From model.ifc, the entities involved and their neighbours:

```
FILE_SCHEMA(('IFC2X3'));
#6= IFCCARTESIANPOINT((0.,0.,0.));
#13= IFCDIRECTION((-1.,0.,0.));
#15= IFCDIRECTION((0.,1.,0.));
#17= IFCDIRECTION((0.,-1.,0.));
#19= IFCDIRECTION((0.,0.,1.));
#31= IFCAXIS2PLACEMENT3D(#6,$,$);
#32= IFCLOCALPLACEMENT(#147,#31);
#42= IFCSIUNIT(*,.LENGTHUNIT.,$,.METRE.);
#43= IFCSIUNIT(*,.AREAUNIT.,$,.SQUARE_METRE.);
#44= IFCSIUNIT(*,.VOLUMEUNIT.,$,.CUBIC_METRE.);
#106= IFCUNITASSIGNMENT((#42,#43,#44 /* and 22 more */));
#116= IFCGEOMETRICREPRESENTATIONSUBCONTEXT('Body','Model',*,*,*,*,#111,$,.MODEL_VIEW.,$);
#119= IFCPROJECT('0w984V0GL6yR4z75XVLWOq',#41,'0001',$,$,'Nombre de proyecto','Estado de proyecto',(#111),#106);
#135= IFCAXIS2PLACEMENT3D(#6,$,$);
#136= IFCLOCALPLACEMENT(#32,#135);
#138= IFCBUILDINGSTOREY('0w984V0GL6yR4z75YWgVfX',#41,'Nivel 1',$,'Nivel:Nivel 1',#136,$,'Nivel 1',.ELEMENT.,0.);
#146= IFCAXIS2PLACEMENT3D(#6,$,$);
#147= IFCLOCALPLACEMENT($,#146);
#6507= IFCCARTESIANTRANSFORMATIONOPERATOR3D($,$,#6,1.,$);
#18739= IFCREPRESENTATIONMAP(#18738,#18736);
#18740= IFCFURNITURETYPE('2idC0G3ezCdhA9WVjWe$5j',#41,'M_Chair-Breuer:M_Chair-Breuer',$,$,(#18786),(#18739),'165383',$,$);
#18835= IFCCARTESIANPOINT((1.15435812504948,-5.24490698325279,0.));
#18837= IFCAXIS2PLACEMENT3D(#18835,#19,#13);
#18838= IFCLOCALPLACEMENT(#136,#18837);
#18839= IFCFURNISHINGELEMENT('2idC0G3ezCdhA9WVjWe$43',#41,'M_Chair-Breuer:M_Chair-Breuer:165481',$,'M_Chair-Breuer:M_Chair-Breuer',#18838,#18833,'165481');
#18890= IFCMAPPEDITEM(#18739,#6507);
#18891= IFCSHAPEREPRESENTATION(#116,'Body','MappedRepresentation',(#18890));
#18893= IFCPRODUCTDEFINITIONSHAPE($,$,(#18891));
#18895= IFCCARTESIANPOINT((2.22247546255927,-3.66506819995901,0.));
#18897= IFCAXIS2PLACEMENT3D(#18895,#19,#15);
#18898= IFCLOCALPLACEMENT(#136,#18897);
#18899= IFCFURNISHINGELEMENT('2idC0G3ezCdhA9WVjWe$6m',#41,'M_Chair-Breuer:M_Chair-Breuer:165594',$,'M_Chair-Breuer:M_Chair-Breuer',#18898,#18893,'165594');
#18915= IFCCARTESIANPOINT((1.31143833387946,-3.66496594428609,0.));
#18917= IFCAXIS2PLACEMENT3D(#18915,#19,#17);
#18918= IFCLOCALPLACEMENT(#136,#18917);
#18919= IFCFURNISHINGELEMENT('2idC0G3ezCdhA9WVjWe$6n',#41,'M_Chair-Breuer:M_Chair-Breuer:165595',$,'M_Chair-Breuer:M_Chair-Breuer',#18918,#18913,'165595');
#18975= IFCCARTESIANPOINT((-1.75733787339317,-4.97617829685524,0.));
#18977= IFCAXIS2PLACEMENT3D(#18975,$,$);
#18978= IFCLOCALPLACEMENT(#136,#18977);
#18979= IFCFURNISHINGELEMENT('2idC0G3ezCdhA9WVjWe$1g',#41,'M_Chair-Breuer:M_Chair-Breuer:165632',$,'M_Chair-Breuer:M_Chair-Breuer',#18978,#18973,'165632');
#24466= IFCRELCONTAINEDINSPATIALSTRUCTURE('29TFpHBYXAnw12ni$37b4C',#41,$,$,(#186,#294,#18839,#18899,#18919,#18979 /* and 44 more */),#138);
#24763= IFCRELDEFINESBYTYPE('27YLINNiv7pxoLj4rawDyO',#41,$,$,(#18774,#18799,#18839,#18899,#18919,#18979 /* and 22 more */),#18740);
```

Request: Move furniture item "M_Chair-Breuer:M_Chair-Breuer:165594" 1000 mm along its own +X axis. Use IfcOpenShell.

```python
import ifcopenshell
import ifcopenshell.api.geometry
import ifcopenshell.util.placement

model = ifcopenshell.open("model.ifc")

item = model.by_guid("2idC0G3ezCdhA9WVjWe$6m")
matrix = ifcopenshell.util.placement.get_local_placement(item.ObjectPlacement)
matrix[:3, 3] += matrix[:3, 0] * 1.0
ifcopenshell.api.geometry.edit_object_placement(model, product=item, matrix=matrix, is_si=False)

print(ifcopenshell.util.placement.get_local_placement(item.ObjectPlacement).round(3) + 0.0)

model.write("model_updated.ifc")
```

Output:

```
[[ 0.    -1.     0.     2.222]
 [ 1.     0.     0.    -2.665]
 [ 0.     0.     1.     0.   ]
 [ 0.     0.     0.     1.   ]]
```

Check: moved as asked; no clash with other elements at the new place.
